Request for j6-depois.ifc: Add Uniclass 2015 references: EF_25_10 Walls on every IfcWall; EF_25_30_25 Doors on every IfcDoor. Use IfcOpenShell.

First a look at what the model holds.

```python
import ifcopenshell

model = ifcopenshell.open("j6-depois.ifc")
print(model.schema)
print("classifications:", [c.Name for c in model.by_type("IfcClassification")])
for ifc_class in ("IfcDoor", "IfcRoof", "IfcStair", "IfcWall", "IfcWindow"):
    print(ifc_class, len(model.by_type(ifc_class)))
```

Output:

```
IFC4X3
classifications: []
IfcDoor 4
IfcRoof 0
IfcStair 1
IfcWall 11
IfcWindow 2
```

```python
import ifcopenshell
import ifcopenshell.api.classification

model = ifcopenshell.open("j6-depois.ifc")

system = ifcopenshell.api.classification.add_classification(model, classification="Uniclass 2015")

codes = {
    "IfcWall": ("EF_25_10", "Walls"),
    "IfcDoor": ("EF_25_30_25", "Doors"),
}
for ifc_class, (code, name) in codes.items():
    products = model.by_type(ifc_class)
    ifcopenshell.api.classification.add_reference(
        model, products=products, classification=system, identification=code, name=name
    )
    print(code, len(products))

model.write("j6-depois-out.ifc")
```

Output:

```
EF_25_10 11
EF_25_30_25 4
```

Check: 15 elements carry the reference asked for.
